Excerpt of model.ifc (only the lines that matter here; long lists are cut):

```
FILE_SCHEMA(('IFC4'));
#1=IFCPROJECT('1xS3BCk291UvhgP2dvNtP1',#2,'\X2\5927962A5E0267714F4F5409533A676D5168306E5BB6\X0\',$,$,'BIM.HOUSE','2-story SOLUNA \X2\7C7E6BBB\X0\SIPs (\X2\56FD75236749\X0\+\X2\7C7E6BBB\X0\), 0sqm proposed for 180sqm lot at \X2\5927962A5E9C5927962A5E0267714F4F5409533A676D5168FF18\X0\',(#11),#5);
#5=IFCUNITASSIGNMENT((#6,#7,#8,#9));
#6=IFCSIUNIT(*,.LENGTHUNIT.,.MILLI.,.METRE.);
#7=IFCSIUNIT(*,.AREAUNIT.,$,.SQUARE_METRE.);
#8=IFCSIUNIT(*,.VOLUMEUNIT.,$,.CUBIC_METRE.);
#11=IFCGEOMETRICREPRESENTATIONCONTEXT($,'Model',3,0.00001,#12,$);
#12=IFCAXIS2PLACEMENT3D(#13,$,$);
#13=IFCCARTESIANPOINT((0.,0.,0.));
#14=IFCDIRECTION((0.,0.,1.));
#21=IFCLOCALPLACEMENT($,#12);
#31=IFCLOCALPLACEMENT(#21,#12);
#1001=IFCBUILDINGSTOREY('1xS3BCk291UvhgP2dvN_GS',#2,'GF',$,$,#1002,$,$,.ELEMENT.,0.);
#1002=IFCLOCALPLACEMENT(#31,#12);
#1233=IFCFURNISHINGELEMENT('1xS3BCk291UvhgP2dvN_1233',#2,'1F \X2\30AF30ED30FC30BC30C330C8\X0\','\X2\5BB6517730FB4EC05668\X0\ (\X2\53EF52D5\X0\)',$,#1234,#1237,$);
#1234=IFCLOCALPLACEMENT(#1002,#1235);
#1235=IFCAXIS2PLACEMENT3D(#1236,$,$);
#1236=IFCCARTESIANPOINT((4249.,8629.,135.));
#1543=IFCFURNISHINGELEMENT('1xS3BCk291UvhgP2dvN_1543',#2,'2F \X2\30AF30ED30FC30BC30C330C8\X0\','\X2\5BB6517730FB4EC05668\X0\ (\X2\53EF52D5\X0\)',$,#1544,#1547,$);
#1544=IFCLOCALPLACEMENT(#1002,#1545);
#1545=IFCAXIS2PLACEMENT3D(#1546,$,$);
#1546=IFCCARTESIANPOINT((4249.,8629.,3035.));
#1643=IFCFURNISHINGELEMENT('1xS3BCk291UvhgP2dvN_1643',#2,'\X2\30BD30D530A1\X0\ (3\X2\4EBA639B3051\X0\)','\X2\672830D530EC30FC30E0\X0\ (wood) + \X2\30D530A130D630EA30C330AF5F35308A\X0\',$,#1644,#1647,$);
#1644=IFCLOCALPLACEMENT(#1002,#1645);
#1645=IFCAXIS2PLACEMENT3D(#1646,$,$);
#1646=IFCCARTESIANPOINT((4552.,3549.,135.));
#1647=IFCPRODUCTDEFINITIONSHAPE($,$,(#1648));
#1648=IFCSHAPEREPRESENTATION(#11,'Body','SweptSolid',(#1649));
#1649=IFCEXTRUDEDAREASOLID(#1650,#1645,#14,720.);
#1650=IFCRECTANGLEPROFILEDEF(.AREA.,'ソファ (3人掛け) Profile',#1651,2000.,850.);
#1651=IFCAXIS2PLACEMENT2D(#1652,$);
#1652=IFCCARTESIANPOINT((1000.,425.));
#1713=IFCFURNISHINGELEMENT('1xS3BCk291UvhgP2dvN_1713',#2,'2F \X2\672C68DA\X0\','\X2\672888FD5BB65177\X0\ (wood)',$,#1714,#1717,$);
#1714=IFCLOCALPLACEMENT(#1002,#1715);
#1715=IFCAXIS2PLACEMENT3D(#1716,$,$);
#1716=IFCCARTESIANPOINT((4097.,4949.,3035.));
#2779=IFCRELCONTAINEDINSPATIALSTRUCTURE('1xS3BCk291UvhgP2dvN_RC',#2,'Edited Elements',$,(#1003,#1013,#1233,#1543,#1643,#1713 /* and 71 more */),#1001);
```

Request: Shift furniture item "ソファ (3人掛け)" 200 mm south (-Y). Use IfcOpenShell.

```python
import ifcopenshell
import ifcopenshell.api.geometry
import ifcopenshell.util.placement
import ifcopenshell.util.unit

model = ifcopenshell.open("model.ifc")
unit_scale = ifcopenshell.util.unit.calculate_unit_scale(model)

item = model.by_guid("1xS3BCk291UvhgP2dvN_1643")
matrix = ifcopenshell.util.placement.get_local_placement(item.ObjectPlacement)
matrix[1, 3] -= 0.2 / unit_scale
ifcopenshell.api.geometry.edit_object_placement(model, product=item, matrix=matrix, is_si=False)

print(ifcopenshell.util.placement.get_local_placement(item.ObjectPlacement).round(3) + 0.0)

model.write("model_edited.ifc")
```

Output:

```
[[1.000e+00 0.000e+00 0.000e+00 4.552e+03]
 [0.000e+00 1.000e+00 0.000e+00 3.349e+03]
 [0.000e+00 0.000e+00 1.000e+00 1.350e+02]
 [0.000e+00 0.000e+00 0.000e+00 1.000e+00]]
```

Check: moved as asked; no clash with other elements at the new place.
